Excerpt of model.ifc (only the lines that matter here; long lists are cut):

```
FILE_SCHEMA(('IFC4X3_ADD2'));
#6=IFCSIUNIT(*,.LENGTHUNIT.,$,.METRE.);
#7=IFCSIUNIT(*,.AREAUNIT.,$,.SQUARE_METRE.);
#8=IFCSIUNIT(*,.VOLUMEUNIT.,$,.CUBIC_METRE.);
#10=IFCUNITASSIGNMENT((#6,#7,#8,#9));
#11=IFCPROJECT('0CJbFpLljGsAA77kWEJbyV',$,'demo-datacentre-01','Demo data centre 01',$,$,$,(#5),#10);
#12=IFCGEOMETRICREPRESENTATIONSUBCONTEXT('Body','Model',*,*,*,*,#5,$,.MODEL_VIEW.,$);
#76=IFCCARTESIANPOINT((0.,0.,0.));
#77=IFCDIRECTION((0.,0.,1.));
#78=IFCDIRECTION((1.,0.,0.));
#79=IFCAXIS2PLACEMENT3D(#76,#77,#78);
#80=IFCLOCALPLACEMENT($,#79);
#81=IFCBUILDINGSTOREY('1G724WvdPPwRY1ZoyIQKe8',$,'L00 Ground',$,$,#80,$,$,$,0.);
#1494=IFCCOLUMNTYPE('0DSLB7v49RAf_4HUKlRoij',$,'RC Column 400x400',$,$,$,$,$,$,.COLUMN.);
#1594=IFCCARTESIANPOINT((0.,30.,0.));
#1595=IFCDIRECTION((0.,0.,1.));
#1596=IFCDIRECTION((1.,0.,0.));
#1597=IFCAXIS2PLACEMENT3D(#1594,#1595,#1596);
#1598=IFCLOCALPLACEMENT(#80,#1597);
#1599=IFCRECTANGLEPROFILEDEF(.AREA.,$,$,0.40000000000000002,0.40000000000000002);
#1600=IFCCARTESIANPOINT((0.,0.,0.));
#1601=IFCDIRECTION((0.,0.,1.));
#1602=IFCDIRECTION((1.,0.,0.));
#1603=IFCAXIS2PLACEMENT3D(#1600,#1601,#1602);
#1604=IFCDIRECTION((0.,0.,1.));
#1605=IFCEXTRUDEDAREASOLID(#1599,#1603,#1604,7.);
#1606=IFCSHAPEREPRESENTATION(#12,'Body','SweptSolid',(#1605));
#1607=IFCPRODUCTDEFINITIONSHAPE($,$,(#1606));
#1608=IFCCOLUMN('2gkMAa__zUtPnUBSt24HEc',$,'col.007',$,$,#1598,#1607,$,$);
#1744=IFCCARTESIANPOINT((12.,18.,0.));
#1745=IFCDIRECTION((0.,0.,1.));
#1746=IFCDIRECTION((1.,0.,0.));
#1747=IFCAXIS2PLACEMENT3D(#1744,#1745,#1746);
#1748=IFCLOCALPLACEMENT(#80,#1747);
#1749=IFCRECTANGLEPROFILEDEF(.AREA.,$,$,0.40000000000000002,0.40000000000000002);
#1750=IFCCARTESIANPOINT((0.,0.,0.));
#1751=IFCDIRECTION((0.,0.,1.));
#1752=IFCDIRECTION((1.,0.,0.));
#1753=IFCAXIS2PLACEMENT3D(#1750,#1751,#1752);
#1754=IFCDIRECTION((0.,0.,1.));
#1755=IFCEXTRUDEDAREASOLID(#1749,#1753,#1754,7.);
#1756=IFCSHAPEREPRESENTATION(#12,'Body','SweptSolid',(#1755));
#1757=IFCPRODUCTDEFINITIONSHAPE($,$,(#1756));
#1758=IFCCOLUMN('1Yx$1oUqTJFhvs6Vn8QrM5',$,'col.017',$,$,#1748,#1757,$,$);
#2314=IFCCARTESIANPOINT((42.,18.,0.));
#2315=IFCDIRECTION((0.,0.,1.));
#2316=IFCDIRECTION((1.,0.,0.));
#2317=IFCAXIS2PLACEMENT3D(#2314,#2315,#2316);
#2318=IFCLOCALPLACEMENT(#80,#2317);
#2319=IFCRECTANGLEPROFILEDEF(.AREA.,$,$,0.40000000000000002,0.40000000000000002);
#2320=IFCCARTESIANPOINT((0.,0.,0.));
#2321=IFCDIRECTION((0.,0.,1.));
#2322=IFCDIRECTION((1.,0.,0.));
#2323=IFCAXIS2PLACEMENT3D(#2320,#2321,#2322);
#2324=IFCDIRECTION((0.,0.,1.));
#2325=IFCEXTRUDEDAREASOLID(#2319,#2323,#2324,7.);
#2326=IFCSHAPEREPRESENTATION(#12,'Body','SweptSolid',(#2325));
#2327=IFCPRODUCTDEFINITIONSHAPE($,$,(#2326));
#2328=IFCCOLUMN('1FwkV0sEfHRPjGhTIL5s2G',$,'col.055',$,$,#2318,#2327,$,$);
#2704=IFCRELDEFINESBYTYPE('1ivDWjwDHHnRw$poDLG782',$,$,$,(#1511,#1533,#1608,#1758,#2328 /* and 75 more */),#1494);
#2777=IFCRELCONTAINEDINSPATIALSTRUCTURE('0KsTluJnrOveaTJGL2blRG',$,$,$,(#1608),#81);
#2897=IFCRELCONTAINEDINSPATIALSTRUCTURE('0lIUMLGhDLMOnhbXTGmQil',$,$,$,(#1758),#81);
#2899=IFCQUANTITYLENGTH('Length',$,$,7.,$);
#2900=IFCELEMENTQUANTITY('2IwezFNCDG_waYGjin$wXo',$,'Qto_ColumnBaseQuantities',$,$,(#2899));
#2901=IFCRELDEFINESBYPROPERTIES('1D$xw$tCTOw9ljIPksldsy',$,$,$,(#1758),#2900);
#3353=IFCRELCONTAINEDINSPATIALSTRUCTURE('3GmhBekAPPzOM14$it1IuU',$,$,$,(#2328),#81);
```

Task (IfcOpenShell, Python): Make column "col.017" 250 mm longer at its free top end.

```python
import ifcopenshell
import ifcopenshell.api.pset
import ifcopenshell.util.element
import ifcopenshell.util.representation
import ifcopenshell.util.unit

model = ifcopenshell.open("model.ifc")
unit_scale = ifcopenshell.util.unit.calculate_unit_scale(model)

member = model.by_guid("1Yx$1oUqTJFhvs6Vn8QrM5")
change = 0.25 / unit_scale

# The extrusion runs towards the end named, so only its depth changes.
body = ifcopenshell.util.representation.get_representation(member, "Model", "Body")
solid = body.Items[0]
old_length = solid.Depth
solid.Depth += change

# Update the stored length and volume.
qto = model.by_id(ifcopenshell.util.element.get_pset(member, "Qto_ColumnBaseQuantities", should_inherit=False)["id"])
ifcopenshell.api.pset.edit_qto(model, qto=qto, properties={"Length": solid.Depth})

print(f"length {old_length:g} -> {solid.Depth:g}")

model.write("model_updated.ifc")
```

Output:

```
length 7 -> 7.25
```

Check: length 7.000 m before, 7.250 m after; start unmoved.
